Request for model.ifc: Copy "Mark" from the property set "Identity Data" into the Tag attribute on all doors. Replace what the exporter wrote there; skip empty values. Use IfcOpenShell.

First a look at what the model holds.

```python
import ifcopenshell
import ifcopenshell.util.element

model = ifcopenshell.open("model.ifc")
print(model.schema)
doors = model.by_type("IfcDoor")
print(len(doors), "doors")
for e in doors[:8]:
    source = ifcopenshell.util.element.get_pset(e, "Identity Data", "Mark")
    target = e.Tag
    print(e.id(), repr(source), repr(target), sep=" | ")
```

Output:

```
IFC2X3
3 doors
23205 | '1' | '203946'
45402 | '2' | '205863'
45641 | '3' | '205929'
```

```python
import ifcopenshell
import ifcopenshell.util.element

model = ifcopenshell.open("model.ifc")

count = 0
for e in model.by_type("IfcDoor"):
    value = ifcopenshell.util.element.get_pset(e, "Identity Data", "Mark")
    current = e.Tag
    if not value or not value.strip() or current == value:
        continue
    e.Tag = value
    count += 1

print(count, "doors updated")

model.write("model-out.ifc")
```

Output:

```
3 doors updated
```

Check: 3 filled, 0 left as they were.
